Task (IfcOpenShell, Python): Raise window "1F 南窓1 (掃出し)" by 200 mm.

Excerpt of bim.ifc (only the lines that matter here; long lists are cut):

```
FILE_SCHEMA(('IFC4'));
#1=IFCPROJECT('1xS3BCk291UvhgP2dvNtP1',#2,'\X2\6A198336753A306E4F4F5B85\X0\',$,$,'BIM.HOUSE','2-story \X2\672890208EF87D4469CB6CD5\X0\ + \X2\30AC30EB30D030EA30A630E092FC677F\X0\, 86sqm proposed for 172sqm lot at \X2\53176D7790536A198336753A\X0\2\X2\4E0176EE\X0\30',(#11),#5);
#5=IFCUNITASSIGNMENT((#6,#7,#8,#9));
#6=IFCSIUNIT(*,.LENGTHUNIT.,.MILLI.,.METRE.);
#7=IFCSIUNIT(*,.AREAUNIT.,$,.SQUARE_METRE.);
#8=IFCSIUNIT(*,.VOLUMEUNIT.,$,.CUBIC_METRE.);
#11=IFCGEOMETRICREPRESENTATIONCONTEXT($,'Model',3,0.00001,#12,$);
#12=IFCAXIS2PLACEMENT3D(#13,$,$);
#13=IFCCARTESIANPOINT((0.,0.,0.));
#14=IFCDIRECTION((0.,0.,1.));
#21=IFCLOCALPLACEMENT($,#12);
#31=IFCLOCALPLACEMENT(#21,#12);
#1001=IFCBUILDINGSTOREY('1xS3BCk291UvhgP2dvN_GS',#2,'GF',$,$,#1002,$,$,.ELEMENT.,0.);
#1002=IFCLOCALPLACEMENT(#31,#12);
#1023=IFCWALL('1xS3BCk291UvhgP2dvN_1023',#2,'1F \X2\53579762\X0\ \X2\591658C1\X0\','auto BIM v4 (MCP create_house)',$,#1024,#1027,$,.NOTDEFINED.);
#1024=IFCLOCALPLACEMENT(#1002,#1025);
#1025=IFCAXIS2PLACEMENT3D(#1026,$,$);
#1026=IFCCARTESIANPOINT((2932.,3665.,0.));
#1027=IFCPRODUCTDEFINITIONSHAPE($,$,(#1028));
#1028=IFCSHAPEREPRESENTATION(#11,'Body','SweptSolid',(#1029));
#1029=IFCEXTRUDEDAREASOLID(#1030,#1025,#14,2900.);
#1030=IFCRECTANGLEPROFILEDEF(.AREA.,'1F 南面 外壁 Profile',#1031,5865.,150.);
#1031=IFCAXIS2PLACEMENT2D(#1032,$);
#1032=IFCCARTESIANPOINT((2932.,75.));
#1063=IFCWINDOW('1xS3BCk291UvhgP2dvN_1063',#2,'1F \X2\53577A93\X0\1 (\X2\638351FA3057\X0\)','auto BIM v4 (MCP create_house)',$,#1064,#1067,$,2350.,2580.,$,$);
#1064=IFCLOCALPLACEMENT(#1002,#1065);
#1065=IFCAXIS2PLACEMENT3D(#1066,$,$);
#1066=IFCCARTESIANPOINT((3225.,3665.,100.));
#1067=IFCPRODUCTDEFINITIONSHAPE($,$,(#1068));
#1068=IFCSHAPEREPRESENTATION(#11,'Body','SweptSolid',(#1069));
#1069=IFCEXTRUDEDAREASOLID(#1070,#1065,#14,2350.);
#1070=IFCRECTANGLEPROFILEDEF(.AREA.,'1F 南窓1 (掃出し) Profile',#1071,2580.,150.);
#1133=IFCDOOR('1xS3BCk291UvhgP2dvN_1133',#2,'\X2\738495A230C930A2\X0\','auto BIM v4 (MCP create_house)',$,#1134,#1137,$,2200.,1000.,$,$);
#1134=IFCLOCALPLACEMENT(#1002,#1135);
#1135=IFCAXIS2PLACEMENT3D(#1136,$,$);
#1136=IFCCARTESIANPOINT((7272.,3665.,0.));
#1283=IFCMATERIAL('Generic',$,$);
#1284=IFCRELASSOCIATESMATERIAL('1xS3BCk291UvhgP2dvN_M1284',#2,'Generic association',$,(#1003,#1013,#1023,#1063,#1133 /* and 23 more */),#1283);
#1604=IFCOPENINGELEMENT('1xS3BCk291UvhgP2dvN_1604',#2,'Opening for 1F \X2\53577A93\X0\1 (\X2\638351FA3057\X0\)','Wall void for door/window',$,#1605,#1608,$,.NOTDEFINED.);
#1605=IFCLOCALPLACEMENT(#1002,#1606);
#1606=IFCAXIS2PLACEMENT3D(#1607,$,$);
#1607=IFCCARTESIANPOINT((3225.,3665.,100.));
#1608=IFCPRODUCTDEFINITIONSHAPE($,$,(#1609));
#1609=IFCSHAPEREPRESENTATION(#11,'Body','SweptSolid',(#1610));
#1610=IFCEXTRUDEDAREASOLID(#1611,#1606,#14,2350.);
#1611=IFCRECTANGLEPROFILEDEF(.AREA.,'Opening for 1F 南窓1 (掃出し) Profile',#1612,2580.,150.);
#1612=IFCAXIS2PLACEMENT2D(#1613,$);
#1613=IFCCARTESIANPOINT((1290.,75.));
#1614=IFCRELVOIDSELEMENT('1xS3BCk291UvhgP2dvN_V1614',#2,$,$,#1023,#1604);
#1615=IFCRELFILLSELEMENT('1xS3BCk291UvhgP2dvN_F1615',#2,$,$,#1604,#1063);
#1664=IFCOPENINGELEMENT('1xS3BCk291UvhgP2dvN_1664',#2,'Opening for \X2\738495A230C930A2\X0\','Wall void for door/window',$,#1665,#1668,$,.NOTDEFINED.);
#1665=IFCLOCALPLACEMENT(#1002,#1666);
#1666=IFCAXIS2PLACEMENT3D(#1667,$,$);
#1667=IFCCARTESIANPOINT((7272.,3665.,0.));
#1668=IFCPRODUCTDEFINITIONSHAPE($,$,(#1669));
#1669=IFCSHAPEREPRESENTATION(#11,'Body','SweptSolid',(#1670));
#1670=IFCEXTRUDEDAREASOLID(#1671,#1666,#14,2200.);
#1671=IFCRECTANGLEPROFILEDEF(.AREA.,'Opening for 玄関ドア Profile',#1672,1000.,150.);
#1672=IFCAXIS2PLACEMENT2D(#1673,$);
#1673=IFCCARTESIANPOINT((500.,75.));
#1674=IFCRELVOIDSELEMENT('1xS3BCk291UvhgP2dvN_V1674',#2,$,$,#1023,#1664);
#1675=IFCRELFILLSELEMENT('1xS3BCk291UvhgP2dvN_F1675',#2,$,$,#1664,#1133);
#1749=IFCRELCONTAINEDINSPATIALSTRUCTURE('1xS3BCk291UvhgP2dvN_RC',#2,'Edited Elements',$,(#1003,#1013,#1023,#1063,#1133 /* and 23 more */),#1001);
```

```python
import numpy as np
import ifcopenshell
import ifcopenshell.api.geometry
import ifcopenshell.util.placement
import ifcopenshell.util.unit

model = ifcopenshell.open("bim.ifc")
unit_scale = ifcopenshell.util.unit.calculate_unit_scale(model)

window = model.by_id(1063)
opening = window.FillsVoids[0].RelatingOpeningElement
dz = 0.2 / unit_scale

shift = np.array([0.0, 0.0, dz])
# The window is not placed relative to its opening, so move both.
for product in (opening, window):
    matrix = ifcopenshell.util.placement.get_local_placement(product.ObjectPlacement)
    matrix[:3, 3] += shift
    ifcopenshell.api.geometry.edit_object_placement(model, product=product, matrix=matrix, is_si=False)

print(f"moved by {dz * unit_scale:+.3f} m")

model.write("bim_v2.ifc")
```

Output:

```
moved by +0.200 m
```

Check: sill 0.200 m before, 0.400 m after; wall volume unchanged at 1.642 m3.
